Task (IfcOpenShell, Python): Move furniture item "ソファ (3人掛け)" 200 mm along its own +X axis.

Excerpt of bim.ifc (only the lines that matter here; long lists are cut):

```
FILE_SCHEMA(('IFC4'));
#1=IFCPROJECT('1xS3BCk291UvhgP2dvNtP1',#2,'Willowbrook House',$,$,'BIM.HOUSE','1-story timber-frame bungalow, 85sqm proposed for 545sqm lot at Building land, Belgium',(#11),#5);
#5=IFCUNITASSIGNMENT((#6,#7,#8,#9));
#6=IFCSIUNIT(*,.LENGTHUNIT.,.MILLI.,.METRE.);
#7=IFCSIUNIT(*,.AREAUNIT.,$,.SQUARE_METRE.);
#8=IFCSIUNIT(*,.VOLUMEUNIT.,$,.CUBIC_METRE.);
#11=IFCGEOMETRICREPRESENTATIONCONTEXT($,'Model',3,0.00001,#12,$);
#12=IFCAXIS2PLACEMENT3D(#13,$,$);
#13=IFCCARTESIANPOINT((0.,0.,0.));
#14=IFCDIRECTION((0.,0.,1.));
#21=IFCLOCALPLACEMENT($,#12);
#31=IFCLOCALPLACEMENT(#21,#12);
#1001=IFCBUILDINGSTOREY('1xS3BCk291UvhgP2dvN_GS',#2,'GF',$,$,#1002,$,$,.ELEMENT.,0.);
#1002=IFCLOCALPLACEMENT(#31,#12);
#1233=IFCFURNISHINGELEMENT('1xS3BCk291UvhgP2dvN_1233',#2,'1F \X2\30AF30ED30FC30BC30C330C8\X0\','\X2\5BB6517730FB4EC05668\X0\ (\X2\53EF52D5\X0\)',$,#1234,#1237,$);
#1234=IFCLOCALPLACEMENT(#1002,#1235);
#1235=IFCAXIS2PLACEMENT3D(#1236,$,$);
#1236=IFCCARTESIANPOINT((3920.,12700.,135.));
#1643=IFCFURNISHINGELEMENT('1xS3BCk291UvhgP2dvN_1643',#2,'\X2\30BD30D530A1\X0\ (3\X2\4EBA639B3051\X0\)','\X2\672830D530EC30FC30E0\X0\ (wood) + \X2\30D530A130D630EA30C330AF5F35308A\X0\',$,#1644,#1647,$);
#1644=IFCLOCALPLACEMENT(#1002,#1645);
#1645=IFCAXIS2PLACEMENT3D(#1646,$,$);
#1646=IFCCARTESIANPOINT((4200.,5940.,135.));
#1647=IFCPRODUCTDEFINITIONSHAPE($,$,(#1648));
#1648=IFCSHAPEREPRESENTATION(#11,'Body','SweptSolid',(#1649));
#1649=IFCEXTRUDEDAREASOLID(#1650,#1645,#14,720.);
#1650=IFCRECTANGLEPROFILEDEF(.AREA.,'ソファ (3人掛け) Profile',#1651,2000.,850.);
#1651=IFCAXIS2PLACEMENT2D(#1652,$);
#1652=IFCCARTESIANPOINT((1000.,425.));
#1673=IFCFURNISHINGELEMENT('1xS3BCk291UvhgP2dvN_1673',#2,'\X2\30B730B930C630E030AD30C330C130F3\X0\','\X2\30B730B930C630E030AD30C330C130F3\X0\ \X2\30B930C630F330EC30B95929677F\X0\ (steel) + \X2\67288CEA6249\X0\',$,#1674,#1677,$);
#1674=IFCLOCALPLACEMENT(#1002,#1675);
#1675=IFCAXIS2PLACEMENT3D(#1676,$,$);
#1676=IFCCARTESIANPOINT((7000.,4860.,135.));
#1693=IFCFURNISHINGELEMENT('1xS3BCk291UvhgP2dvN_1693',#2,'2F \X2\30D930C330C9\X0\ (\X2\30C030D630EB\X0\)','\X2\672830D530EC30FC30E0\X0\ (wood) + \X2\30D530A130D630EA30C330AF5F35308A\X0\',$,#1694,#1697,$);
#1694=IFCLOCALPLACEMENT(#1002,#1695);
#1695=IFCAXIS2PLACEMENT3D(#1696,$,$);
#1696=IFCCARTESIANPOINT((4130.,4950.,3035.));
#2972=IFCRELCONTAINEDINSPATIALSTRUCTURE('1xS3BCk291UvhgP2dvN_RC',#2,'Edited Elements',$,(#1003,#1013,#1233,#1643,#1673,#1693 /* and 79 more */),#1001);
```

```python
import ifcopenshell
import ifcopenshell.api.geometry
import ifcopenshell.util.placement
import ifcopenshell.util.unit

model = ifcopenshell.open("bim.ifc")
unit_scale = ifcopenshell.util.unit.calculate_unit_scale(model)

item = model.by_id(1643)
matrix = ifcopenshell.util.placement.get_local_placement(item.ObjectPlacement)
matrix[:3, 3] += matrix[:3, 0] * 0.2 / unit_scale
ifcopenshell.api.geometry.edit_object_placement(model, product=item, matrix=matrix, is_si=False)

print(ifcopenshell.util.placement.get_local_placement(item.ObjectPlacement).round(3) + 0.0)

model.write("bim-out.ifc")
```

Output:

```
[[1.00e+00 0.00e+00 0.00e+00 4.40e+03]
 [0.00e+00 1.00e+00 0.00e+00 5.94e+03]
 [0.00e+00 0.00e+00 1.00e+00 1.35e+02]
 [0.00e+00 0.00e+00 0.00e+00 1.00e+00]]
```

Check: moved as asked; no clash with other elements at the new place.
